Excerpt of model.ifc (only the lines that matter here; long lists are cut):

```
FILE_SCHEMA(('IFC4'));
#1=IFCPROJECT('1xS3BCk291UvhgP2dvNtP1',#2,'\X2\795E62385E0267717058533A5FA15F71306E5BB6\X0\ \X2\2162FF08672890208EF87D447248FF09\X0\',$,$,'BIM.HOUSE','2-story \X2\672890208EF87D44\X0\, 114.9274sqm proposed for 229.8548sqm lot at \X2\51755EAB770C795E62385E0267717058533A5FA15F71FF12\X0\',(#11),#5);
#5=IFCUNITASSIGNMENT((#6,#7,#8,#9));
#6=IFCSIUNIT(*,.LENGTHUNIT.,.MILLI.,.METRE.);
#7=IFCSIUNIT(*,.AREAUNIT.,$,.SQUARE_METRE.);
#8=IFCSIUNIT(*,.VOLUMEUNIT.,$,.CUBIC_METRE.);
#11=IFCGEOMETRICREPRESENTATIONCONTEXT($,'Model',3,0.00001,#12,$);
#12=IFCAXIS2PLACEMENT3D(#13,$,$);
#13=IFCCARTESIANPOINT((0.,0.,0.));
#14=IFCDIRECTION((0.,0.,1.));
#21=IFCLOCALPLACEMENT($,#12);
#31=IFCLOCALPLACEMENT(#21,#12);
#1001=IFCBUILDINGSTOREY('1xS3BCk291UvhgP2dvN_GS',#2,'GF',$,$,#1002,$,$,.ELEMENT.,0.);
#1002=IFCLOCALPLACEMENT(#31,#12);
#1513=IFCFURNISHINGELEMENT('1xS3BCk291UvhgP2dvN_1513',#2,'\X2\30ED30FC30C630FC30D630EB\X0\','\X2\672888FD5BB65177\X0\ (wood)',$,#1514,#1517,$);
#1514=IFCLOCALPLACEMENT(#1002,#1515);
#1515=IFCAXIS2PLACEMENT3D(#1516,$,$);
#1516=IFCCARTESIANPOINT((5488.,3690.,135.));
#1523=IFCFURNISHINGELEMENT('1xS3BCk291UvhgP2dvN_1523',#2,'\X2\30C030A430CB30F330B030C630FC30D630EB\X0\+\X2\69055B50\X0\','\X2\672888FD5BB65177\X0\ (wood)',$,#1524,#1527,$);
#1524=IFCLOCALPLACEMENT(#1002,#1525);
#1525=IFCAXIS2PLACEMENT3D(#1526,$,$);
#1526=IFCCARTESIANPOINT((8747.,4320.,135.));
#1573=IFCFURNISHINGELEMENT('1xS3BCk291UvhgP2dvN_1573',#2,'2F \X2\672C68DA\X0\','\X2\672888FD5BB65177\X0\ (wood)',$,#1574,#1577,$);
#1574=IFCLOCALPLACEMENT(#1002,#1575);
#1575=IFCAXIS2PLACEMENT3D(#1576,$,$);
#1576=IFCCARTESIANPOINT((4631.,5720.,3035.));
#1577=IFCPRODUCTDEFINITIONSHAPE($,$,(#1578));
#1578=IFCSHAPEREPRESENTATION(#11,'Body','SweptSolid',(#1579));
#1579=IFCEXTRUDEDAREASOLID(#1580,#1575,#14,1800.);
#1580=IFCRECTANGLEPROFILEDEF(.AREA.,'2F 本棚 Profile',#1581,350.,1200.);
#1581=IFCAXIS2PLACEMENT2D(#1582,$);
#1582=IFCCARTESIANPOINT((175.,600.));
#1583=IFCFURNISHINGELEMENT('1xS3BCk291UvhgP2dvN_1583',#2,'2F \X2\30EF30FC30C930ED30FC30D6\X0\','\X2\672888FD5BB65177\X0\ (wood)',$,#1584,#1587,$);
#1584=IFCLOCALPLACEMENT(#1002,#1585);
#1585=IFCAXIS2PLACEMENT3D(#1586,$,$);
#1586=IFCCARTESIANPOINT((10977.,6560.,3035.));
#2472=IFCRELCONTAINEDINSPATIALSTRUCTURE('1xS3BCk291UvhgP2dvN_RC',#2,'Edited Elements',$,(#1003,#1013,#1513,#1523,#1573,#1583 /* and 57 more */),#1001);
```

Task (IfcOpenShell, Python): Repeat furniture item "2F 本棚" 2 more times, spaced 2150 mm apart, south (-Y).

```python
import numpy as np
import ifcopenshell
import ifcopenshell.api.geometry
import ifcopenshell.api.root
import ifcopenshell.util.element
import ifcopenshell.util.placement
import ifcopenshell.util.unit

model = ifcopenshell.open("model.ifc")
unit_scale = ifcopenshell.util.unit.calculate_unit_scale(model)


def reuse_history(source, copy):
    """copy_class also copies each property set's owner history, people and application; keep the originals."""
    for rel in copy.IsDefinedBy:
        if rel.is_a("IfcRelDefinesByProperties") and (history := rel.RelatingPropertyDefinition.OwnerHistory):
            rel.RelatingPropertyDefinition.OwnerHistory = source.OwnerHistory
            ifcopenshell.util.element.remove_deep2(model, history)


source = model.by_id(1573)
base = ifcopenshell.util.placement.get_local_placement(source.ObjectPlacement)
step = np.array([0.0, -1.0, 0.0]) * 2.15 / unit_scale

for i in range(1, 3):
    copy = ifcopenshell.api.root.copy_class(model, product=source)
    copy.Representation = ifcopenshell.util.element.copy_deep(
        model, source.Representation, exclude=["IfcGeometricRepresentationContext", "IfcRepresentationMap"]
    )
    reuse_history(source, copy)
    matrix = base.copy()
    matrix[:3, 3] += i * step
    print("added at", matrix[:3, 3].round(3) + 0.0)
    ifcopenshell.api.geometry.edit_object_placement(model, product=copy, matrix=matrix, is_si=False)

model.write("model_rev.ifc")
```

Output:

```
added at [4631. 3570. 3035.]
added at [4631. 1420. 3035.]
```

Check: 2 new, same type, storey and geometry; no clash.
